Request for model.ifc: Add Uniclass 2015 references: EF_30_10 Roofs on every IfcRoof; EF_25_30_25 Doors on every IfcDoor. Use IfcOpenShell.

First a look at what the model holds.

```python
import ifcopenshell

model = ifcopenshell.open("model.ifc")
print(model.schema)
print("classifications:", [c.Name for c in model.by_type("IfcClassification")])
for ifc_class in ("IfcDoor", "IfcRoof", "IfcStair", "IfcWall", "IfcWindow"):
    print(ifc_class, len(model.by_type(ifc_class)))
```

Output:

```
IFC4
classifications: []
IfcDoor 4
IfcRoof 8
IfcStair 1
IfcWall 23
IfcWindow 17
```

```python
import ifcopenshell
import ifcopenshell.api.classification

model = ifcopenshell.open("model.ifc")

system = ifcopenshell.api.classification.add_classification(model, classification="Uniclass 2015")

codes = {
    "IfcRoof": ("EF_30_10", "Roofs"),
    "IfcDoor": ("EF_25_30_25", "Doors"),
}
for ifc_class, (code, name) in codes.items():
    products = model.by_type(ifc_class)
    ifcopenshell.api.classification.add_reference(
        model, products=products, classification=system, identification=code, name=name
    )
    print(code, len(products))

model.write("model_v2.ifc")
```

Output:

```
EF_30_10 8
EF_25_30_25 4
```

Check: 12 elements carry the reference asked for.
